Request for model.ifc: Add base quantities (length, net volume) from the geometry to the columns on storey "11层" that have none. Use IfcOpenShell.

First a look at what the model holds.

```python
import ifcopenshell
import ifcopenshell.util.element
import ifcopenshell.util.unit

model = ifcopenshell.open("model.ifc")
print(model.schema)
for unit_type in ("LENGTHUNIT", "AREAUNIT", "VOLUMEUNIT"):
    print(unit_type, ifcopenshell.util.unit.calculate_unit_scale(model, unit_type))
storey = next(s for s in model.by_type("IfcBuildingStorey") if s.Name == "11层")
columns = [e for e in ifcopenshell.util.element.get_decomposition(storey) if e.is_a("IfcColumn")]
for e in sorted(columns, key=lambda e: e.id()):
    print(e.id(), e.is_a(), e.Name, list(ifcopenshell.util.element.get_psets(e, qtos_only=True)), sep=" | ")
```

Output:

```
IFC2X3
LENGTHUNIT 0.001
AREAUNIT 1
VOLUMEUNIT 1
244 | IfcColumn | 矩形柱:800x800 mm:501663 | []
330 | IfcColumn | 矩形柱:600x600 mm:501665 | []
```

```python
import ifcopenshell
import ifcopenshell.api.pset
import ifcopenshell.geom
import ifcopenshell.util.element
import ifcopenshell.util.shape
import ifcopenshell.util.unit

model = ifcopenshell.open("model.ifc")
unit_scale = ifcopenshell.util.unit.calculate_unit_scale(model)
volume_scale = ifcopenshell.util.unit.calculate_unit_scale(model, "VOLUMEUNIT")
settings = ifcopenshell.geom.settings()

storey = next(s for s in model.by_type("IfcBuildingStorey") if s.Name == "11层")
columns = [e for e in ifcopenshell.util.element.get_decomposition(storey) if e.is_a("IfcColumn")]

for e in sorted(columns, key=lambda e: e.id()):
    if ifcopenshell.util.element.get_psets(e, qtos_only=True, should_inherit=False):
        continue
    # Geometry comes back in metres, in the element's own axes.
    shape = ifcopenshell.geom.create_shape(settings, e)
    values = {
        "Length": ifcopenshell.util.shape.get_z(shape.geometry) / unit_scale,
        "NetVolume": ifcopenshell.util.shape.get_volume(shape.geometry) / volume_scale,
    }
    qto = ifcopenshell.api.pset.add_qto(model, product=e, name="BaseQuantities")
    ifcopenshell.api.pset.edit_qto(model, qto=qto, properties=values)
    print(e.id(), {k: round(v, 3) for k, v in values.items()})

model.write("model_v2.ifc")
```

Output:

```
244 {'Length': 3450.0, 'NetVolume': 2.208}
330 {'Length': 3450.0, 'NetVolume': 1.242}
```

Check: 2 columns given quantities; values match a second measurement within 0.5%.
